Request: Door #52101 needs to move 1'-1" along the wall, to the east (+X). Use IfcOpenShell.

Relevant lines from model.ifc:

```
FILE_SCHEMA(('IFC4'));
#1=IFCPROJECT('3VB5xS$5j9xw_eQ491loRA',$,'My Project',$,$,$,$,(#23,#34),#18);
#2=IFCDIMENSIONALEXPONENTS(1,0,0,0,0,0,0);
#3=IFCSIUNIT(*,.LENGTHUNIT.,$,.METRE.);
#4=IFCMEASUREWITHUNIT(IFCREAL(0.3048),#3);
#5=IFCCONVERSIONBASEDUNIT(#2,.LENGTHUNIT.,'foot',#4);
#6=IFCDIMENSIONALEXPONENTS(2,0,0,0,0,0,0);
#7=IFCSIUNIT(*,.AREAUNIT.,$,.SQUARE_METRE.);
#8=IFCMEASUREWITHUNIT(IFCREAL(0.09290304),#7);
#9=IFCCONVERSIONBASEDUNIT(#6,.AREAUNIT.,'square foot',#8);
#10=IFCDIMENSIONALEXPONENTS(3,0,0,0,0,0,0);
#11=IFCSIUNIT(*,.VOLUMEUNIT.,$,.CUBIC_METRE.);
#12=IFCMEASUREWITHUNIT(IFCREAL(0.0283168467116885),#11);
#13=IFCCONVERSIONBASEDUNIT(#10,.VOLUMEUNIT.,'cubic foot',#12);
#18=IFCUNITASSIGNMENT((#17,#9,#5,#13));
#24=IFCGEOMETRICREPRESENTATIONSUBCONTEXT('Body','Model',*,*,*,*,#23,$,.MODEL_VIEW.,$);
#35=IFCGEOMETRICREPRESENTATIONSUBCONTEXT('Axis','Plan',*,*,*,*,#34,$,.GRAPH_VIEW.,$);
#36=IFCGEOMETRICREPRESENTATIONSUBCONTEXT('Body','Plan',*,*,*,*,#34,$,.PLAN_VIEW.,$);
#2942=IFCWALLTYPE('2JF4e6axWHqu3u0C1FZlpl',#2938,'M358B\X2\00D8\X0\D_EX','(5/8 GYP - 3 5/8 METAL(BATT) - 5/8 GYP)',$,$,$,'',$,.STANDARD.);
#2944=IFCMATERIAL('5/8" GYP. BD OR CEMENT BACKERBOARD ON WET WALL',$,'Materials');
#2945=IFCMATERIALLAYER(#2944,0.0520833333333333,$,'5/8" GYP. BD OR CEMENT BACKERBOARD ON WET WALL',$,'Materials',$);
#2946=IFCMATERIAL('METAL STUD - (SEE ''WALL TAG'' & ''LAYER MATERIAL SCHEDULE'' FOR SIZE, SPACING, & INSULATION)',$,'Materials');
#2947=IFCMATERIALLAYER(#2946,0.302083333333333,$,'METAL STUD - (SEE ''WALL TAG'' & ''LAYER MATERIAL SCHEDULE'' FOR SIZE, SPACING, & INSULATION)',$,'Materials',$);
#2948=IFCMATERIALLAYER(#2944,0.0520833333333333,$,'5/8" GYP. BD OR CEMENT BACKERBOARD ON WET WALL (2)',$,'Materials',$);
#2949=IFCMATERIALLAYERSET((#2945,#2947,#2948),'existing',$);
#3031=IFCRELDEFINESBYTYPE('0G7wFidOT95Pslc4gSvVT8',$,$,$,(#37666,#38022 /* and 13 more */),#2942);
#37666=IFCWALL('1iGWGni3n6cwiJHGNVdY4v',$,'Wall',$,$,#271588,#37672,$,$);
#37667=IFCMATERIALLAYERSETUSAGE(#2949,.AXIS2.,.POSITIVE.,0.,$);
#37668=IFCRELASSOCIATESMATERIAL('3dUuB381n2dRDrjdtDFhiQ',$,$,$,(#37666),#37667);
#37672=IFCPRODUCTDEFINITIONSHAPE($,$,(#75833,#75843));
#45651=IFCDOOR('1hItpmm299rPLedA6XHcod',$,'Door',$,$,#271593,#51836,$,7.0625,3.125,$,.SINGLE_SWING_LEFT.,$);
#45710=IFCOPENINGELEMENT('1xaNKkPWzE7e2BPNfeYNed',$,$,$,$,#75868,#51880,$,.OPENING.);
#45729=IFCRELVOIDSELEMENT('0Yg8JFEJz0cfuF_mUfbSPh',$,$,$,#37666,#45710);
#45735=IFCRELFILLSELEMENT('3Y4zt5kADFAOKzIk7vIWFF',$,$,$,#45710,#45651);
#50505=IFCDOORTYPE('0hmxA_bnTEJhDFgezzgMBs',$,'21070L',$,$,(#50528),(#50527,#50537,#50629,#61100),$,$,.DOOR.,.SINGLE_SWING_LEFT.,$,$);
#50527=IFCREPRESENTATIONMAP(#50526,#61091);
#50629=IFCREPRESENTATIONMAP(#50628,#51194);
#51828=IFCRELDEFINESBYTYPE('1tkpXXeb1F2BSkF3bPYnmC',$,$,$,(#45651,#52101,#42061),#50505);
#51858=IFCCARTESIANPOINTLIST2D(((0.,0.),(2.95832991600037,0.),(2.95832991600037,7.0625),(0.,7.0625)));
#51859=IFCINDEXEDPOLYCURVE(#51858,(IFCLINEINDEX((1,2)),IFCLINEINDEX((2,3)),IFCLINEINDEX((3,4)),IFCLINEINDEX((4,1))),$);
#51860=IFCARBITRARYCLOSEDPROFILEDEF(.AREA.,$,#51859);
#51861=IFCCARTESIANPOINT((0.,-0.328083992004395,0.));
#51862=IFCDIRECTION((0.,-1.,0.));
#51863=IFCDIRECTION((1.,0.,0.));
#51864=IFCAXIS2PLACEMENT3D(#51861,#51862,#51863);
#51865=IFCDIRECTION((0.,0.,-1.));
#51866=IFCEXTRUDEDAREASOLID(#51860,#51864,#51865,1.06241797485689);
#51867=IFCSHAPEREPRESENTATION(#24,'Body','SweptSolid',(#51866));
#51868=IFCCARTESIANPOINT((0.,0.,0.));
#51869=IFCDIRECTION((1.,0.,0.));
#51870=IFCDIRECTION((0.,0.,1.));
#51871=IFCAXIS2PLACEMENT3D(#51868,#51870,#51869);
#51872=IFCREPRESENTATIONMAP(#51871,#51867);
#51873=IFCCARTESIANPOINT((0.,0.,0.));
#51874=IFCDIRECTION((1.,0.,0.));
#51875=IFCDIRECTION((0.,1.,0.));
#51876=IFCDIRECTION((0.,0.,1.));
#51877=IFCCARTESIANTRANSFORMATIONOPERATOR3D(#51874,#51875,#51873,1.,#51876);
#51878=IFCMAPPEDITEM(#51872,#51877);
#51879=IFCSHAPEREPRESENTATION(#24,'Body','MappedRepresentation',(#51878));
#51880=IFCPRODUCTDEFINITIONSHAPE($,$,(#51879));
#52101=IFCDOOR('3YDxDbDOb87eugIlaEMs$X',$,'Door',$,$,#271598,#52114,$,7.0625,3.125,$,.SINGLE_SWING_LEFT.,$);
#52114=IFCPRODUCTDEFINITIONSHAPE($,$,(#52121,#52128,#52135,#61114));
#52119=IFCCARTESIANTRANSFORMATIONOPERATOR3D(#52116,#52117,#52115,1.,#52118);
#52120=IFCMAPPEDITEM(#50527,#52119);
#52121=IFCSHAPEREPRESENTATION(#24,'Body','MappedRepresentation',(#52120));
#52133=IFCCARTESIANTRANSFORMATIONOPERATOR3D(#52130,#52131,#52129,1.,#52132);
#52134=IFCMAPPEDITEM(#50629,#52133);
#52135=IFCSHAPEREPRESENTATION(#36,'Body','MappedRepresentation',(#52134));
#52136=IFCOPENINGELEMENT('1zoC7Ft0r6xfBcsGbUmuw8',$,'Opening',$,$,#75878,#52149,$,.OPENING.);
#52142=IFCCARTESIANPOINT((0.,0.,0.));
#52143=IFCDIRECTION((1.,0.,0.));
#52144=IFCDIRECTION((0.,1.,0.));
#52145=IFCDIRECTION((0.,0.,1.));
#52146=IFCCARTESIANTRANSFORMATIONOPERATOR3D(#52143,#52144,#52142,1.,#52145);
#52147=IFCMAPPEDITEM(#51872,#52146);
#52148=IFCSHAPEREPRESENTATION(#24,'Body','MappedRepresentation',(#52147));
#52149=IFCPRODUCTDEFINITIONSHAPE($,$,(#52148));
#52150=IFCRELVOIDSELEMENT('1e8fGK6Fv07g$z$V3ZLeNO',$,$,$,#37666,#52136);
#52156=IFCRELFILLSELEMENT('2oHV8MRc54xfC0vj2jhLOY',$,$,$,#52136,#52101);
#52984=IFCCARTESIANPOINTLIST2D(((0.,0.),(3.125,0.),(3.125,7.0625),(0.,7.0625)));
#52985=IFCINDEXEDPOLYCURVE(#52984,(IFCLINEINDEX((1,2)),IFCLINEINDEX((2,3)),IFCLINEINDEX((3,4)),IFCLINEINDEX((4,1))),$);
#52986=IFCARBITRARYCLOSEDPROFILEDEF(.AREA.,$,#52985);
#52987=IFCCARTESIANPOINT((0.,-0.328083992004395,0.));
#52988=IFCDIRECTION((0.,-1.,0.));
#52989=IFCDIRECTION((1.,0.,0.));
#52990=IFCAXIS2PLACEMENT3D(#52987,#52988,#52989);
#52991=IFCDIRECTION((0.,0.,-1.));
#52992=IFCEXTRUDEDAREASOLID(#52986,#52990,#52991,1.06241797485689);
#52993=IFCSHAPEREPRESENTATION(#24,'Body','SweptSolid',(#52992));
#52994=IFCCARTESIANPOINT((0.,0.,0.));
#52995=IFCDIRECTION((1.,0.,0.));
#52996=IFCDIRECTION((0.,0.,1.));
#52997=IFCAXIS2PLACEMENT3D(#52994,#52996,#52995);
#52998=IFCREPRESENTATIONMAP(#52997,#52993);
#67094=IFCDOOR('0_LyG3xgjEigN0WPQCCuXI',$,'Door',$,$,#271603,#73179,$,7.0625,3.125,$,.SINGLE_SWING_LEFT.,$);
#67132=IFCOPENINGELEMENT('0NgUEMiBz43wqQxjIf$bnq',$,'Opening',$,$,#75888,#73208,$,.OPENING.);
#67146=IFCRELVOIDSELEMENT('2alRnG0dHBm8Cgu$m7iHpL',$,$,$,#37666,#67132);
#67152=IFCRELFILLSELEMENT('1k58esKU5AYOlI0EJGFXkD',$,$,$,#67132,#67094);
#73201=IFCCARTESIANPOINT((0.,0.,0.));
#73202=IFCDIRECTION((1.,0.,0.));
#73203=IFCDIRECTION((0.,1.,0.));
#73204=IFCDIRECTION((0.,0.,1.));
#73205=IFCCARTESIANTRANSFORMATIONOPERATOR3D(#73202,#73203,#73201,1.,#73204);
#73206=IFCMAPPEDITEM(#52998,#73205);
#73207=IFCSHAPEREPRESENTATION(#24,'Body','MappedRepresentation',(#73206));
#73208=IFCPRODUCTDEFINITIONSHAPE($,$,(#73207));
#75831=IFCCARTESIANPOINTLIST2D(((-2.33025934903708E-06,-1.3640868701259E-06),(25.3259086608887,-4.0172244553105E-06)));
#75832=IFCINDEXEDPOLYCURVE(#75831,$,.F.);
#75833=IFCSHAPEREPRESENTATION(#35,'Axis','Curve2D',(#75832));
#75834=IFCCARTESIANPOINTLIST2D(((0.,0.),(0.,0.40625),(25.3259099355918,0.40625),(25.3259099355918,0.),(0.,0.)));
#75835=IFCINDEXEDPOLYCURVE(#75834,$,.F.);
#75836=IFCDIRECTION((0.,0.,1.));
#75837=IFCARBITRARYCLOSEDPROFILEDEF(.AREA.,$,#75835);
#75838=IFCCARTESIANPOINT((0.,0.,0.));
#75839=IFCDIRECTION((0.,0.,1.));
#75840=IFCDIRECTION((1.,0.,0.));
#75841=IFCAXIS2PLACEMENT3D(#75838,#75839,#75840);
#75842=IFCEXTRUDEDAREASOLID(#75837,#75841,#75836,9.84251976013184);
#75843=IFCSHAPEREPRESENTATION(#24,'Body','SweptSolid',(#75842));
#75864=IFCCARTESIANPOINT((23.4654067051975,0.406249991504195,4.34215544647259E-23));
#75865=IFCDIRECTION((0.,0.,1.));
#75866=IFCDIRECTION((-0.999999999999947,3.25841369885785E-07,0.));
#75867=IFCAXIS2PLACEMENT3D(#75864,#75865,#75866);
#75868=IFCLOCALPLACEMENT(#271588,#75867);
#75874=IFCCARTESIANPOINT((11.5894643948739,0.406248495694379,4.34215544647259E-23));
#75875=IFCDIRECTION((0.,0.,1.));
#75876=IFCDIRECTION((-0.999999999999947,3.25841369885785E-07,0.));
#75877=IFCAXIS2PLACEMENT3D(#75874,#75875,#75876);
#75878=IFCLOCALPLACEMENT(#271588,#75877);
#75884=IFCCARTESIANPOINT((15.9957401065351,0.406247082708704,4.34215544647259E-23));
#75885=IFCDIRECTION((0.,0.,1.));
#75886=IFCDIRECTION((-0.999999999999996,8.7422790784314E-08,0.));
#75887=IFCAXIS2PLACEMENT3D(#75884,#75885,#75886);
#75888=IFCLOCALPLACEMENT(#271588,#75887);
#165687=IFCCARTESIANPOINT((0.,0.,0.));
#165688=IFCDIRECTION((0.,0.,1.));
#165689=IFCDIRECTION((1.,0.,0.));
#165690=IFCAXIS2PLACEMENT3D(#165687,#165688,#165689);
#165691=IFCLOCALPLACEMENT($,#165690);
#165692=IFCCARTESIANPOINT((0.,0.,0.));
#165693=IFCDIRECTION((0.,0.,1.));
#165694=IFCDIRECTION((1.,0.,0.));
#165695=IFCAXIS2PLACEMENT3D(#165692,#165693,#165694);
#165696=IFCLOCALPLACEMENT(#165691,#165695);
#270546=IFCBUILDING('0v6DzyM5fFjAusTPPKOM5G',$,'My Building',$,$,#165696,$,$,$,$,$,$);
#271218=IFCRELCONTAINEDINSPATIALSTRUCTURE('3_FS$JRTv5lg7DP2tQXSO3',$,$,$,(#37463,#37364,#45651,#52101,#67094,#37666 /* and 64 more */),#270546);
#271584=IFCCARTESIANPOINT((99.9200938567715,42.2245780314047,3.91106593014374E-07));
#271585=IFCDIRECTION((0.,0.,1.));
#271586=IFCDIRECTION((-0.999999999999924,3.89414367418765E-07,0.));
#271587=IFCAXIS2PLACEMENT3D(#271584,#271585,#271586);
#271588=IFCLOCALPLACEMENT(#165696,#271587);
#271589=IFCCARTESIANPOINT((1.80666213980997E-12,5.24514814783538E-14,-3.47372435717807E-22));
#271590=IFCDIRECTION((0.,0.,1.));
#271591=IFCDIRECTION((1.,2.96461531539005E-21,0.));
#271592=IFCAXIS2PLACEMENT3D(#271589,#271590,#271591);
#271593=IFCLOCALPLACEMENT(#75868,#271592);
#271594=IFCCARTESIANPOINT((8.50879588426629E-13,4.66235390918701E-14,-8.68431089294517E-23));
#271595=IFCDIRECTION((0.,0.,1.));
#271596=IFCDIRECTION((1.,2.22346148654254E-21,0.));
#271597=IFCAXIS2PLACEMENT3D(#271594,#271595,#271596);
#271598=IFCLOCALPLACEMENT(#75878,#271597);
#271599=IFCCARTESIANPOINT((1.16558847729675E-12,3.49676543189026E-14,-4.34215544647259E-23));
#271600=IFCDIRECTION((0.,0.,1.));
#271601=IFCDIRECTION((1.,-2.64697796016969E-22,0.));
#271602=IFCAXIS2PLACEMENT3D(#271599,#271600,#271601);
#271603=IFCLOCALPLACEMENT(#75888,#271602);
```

```python
import ifcopenshell
import ifcopenshell.api.geometry
import ifcopenshell.util.placement
import ifcopenshell.util.unit

model = ifcopenshell.open("model.ifc")
unit_scale = ifcopenshell.util.unit.calculate_unit_scale(model)

door = model.by_guid("3YDxDbDOb87eugIlaEMs$X")
opening = door.FillsVoids[0].RelatingOpeningElement
wall = opening.VoidsElements[0].RelatingBuildingElement

wall_matrix = ifcopenshell.util.placement.get_local_placement(wall.ObjectPlacement)
shift = wall_matrix[:3, 0] * -13 * 0.0254 / unit_scale
before = ifcopenshell.util.placement.get_local_placement(door.ObjectPlacement)[:3, 3].copy()

# The door is placed relative to its opening, so it follows when the opening moves.
matrix = ifcopenshell.util.placement.get_local_placement(opening.ObjectPlacement)
matrix[:3, 3] += shift
ifcopenshell.api.geometry.edit_object_placement(
    model, product=opening, matrix=matrix, is_si=False, should_transform_children=True
)

after = ifcopenshell.util.placement.get_local_placement(door.ObjectPlacement)[:3, 3]
print("door moved by", (after - before).round(3) + 0.0)

model.write("model-out.ifc")
```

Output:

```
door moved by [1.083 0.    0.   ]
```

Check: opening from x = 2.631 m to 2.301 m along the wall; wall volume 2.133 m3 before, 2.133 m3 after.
